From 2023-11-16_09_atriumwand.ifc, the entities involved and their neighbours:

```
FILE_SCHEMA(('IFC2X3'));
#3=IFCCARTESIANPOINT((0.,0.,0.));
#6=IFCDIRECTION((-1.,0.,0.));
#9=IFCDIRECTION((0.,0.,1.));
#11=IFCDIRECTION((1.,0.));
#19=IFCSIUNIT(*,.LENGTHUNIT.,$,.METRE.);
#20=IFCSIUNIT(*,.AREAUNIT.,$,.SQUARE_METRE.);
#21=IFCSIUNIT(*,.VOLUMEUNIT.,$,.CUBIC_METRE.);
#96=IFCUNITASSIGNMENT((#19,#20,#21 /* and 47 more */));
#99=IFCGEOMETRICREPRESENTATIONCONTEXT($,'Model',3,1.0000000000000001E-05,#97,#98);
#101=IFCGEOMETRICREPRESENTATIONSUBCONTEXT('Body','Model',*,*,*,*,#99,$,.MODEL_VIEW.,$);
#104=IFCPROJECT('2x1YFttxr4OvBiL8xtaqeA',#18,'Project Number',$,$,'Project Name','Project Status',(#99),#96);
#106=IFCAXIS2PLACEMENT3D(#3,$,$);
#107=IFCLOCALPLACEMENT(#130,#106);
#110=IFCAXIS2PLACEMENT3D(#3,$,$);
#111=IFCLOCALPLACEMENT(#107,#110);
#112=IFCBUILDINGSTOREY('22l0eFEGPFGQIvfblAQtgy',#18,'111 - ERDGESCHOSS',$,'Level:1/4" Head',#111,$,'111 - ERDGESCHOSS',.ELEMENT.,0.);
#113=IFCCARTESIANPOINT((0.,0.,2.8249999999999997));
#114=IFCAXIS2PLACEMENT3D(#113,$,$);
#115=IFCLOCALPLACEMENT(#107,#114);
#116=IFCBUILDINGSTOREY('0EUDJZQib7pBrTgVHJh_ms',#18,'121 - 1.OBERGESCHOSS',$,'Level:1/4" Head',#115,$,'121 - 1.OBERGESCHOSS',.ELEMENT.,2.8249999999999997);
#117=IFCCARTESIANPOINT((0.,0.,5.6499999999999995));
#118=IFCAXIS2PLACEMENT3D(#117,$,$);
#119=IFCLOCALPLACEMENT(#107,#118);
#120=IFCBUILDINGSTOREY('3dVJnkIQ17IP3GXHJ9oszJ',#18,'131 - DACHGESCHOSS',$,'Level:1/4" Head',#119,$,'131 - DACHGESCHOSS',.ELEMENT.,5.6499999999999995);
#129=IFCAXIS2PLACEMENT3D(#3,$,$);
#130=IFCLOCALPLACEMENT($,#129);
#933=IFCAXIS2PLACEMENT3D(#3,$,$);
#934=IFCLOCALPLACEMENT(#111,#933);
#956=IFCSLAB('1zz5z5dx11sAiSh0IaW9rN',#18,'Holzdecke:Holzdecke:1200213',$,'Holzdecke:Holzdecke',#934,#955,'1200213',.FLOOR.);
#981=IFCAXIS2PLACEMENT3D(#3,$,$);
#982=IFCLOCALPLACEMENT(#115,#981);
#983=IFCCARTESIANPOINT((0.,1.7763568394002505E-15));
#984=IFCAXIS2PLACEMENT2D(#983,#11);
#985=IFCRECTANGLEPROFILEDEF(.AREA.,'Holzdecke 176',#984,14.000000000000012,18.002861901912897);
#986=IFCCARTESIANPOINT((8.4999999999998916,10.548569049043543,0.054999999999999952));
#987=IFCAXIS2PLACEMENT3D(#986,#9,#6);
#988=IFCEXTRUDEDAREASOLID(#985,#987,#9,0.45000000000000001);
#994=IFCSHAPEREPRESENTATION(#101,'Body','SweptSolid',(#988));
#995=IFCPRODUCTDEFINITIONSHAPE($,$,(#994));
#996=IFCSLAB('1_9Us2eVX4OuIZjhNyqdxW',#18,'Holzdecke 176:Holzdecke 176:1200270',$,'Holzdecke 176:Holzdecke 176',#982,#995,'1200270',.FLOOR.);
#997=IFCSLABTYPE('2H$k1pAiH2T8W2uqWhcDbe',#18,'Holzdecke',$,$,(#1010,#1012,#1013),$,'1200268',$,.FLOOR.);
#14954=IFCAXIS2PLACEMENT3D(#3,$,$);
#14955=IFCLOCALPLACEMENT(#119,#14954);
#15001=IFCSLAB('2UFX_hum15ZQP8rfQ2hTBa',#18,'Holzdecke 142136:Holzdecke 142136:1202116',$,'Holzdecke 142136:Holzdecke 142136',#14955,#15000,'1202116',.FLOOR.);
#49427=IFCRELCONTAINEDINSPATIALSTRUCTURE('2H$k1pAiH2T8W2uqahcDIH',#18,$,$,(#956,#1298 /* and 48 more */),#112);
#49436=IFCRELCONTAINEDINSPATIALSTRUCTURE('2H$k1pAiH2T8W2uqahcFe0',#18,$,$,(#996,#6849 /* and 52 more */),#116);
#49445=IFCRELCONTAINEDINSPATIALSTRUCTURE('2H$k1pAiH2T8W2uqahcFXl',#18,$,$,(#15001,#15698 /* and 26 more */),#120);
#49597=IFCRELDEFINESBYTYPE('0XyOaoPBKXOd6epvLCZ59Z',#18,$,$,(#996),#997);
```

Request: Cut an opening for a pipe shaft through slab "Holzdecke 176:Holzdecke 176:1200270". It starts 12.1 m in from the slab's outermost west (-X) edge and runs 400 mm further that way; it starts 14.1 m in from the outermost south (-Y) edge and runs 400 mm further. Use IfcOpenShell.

```python
import numpy as np
import ifcopenshell
import ifcopenshell.api.feature
import ifcopenshell.api.geometry
import ifcopenshell.api.root
import ifcopenshell.geom
import ifcopenshell.util.placement
import ifcopenshell.util.representation
import ifcopenshell.util.shape
import ifcopenshell.util.unit

model = ifcopenshell.open("2023-11-16_09_atriumwand.ifc")
unit_scale = ifcopenshell.util.unit.calculate_unit_scale(model)
settings = ifcopenshell.geom.settings()


def volume(element):
    """Net volume in cubic metres, openings subtracted."""
    shape = ifcopenshell.geom.create_shape(settings, element)
    return ifcopenshell.util.shape.get_volume(shape.geometry)


slab = model.by_guid("1_9Us2eVX4OuIZjhNyqdxW")
before = volume(slab)

# Extent in the slab's own axes, in metres. The edges named are its -X and -Y sides.
slab_shape = ifcopenshell.geom.create_shape(settings, slab)
vertices = ifcopenshell.util.shape.get_vertices(slab_shape.geometry)
x_min, y_min, bottom = vertices.min(axis=0)
top = vertices[:, 2].max()

opening = ifcopenshell.api.root.create_entity(model, ifc_class="IfcOpeningElement", name="Pipe shaft opening")
context = ifcopenshell.util.representation.get_context(model, "Model", "Body", "MODEL_VIEW")
width, depth = 0.4, 0.4
outline = [(0.0, 0.0), (width, 0.0), (width, depth), (0.0, depth), (0.0, 0.0)]
# Overshoot both faces by 50 mm so the cut is clean.
shape = ifcopenshell.api.geometry.add_slab_representation(
    model, context=context, depth=top - bottom + 0.1, polyline=outline
)
ifcopenshell.api.geometry.assign_representation(model, product=opening, representation=shape)

matrix = ifcopenshell.util.placement.get_local_placement(slab.ObjectPlacement)
matrix[:, 3] = matrix @ np.append(np.array([x_min + 12.1, y_min + 14.1, bottom - 0.05]) / unit_scale, 1.0)
ifcopenshell.api.geometry.edit_object_placement(model, product=opening, matrix=matrix, is_si=False)
ifcopenshell.api.feature.add_feature(model, feature=opening, element=slab)

after = volume(slab)

print(f"slab volume {before:.3f} -> {after:.3f} m3")

model.write("2023-11-16_09_atriumwand_updated.ifc")
```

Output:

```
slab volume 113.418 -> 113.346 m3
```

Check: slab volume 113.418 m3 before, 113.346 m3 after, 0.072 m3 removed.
